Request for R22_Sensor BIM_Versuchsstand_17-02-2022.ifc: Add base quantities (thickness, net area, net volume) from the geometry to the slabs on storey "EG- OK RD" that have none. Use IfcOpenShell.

First a look at what the model holds.

```python
import ifcopenshell
import ifcopenshell.util.element
import ifcopenshell.util.unit

model = ifcopenshell.open("R22_Sensor BIM_Versuchsstand_17-02-2022.ifc")
print(model.schema)
for unit_type in ("LENGTHUNIT", "AREAUNIT", "VOLUMEUNIT"):
    print(unit_type, ifcopenshell.util.unit.calculate_unit_scale(model, unit_type))
storey = next(s for s in model.by_type("IfcBuildingStorey") if s.Name == "EG- OK RD")
slabs = [e for e in ifcopenshell.util.element.get_decomposition(storey) if e.is_a("IfcSlab")]
for e in sorted(slabs, key=lambda e: e.id()):
    print(e.id(), e.is_a(), e.Name, list(ifcopenshell.util.element.get_psets(e, qtos_only=True)), sep=" | ")
```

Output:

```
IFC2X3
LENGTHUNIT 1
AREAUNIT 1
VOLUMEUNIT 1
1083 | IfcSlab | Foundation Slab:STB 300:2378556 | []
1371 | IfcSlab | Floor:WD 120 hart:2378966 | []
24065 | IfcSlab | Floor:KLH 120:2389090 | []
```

```python
import ifcopenshell
import ifcopenshell.api.pset
import ifcopenshell.geom
import ifcopenshell.util.element
import ifcopenshell.util.shape
import ifcopenshell.util.unit

model = ifcopenshell.open("R22_Sensor BIM_Versuchsstand_17-02-2022.ifc")
unit_scale = ifcopenshell.util.unit.calculate_unit_scale(model)
area_scale = ifcopenshell.util.unit.calculate_unit_scale(model, "AREAUNIT")
volume_scale = ifcopenshell.util.unit.calculate_unit_scale(model, "VOLUMEUNIT")
settings = ifcopenshell.geom.settings()

storey = next(s for s in model.by_type("IfcBuildingStorey") if s.Name == "EG- OK RD")
slabs = [e for e in ifcopenshell.util.element.get_decomposition(storey) if e.is_a("IfcSlab")]

for e in sorted(slabs, key=lambda e: e.id()):
    if ifcopenshell.util.element.get_psets(e, qtos_only=True, should_inherit=False):
        continue
    # Geometry comes back in metres, in the element's own axes.
    shape = ifcopenshell.geom.create_shape(settings, e)
    values = {
        "Width": ifcopenshell.util.shape.get_z(shape.geometry) / unit_scale,
        "NetArea": ifcopenshell.util.shape.get_footprint_area(shape.geometry) / area_scale,
        "NetVolume": ifcopenshell.util.shape.get_volume(shape.geometry) / volume_scale,
    }
    qto = ifcopenshell.api.pset.add_qto(model, product=e, name="BaseQuantities")
    ifcopenshell.api.pset.edit_qto(model, qto=qto, properties=values)
    print(e.id(), {k: round(v, 3) for k, v in values.items()})

model.write("R22_Sensor BIM_Versuchsstand_17-02-2022_v2.ifc")
```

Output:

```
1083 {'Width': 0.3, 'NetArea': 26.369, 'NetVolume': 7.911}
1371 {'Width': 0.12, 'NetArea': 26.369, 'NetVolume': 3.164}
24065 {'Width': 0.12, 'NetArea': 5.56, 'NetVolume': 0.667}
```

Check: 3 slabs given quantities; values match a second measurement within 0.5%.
